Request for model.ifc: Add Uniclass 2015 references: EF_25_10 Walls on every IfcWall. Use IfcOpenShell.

First a look at what the model holds.

```python
import ifcopenshell

model = ifcopenshell.open("model.ifc")
print(model.schema)
print("classifications:", [c.Name for c in model.by_type("IfcClassification")])
for ifc_class in ("IfcDoor", "IfcRoof", "IfcStair", "IfcWall", "IfcWindow"):
    print(ifc_class, len(model.by_type(ifc_class)))
```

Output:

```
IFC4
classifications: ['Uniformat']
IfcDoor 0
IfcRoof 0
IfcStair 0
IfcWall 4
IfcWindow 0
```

```python
import ifcopenshell
import ifcopenshell.api.classification

model = ifcopenshell.open("model.ifc")

system = ifcopenshell.api.classification.add_classification(model, classification="Uniclass 2015")

codes = {
    "IfcWall": ("EF_25_10", "Walls"),
}
for ifc_class, (code, name) in codes.items():
    products = model.by_type(ifc_class)
    ifcopenshell.api.classification.add_reference(
        model, products=products, classification=system, identification=code, name=name
    )
    print(code, len(products))

model.write("model_updated.ifc")
```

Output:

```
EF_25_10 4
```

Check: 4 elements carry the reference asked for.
